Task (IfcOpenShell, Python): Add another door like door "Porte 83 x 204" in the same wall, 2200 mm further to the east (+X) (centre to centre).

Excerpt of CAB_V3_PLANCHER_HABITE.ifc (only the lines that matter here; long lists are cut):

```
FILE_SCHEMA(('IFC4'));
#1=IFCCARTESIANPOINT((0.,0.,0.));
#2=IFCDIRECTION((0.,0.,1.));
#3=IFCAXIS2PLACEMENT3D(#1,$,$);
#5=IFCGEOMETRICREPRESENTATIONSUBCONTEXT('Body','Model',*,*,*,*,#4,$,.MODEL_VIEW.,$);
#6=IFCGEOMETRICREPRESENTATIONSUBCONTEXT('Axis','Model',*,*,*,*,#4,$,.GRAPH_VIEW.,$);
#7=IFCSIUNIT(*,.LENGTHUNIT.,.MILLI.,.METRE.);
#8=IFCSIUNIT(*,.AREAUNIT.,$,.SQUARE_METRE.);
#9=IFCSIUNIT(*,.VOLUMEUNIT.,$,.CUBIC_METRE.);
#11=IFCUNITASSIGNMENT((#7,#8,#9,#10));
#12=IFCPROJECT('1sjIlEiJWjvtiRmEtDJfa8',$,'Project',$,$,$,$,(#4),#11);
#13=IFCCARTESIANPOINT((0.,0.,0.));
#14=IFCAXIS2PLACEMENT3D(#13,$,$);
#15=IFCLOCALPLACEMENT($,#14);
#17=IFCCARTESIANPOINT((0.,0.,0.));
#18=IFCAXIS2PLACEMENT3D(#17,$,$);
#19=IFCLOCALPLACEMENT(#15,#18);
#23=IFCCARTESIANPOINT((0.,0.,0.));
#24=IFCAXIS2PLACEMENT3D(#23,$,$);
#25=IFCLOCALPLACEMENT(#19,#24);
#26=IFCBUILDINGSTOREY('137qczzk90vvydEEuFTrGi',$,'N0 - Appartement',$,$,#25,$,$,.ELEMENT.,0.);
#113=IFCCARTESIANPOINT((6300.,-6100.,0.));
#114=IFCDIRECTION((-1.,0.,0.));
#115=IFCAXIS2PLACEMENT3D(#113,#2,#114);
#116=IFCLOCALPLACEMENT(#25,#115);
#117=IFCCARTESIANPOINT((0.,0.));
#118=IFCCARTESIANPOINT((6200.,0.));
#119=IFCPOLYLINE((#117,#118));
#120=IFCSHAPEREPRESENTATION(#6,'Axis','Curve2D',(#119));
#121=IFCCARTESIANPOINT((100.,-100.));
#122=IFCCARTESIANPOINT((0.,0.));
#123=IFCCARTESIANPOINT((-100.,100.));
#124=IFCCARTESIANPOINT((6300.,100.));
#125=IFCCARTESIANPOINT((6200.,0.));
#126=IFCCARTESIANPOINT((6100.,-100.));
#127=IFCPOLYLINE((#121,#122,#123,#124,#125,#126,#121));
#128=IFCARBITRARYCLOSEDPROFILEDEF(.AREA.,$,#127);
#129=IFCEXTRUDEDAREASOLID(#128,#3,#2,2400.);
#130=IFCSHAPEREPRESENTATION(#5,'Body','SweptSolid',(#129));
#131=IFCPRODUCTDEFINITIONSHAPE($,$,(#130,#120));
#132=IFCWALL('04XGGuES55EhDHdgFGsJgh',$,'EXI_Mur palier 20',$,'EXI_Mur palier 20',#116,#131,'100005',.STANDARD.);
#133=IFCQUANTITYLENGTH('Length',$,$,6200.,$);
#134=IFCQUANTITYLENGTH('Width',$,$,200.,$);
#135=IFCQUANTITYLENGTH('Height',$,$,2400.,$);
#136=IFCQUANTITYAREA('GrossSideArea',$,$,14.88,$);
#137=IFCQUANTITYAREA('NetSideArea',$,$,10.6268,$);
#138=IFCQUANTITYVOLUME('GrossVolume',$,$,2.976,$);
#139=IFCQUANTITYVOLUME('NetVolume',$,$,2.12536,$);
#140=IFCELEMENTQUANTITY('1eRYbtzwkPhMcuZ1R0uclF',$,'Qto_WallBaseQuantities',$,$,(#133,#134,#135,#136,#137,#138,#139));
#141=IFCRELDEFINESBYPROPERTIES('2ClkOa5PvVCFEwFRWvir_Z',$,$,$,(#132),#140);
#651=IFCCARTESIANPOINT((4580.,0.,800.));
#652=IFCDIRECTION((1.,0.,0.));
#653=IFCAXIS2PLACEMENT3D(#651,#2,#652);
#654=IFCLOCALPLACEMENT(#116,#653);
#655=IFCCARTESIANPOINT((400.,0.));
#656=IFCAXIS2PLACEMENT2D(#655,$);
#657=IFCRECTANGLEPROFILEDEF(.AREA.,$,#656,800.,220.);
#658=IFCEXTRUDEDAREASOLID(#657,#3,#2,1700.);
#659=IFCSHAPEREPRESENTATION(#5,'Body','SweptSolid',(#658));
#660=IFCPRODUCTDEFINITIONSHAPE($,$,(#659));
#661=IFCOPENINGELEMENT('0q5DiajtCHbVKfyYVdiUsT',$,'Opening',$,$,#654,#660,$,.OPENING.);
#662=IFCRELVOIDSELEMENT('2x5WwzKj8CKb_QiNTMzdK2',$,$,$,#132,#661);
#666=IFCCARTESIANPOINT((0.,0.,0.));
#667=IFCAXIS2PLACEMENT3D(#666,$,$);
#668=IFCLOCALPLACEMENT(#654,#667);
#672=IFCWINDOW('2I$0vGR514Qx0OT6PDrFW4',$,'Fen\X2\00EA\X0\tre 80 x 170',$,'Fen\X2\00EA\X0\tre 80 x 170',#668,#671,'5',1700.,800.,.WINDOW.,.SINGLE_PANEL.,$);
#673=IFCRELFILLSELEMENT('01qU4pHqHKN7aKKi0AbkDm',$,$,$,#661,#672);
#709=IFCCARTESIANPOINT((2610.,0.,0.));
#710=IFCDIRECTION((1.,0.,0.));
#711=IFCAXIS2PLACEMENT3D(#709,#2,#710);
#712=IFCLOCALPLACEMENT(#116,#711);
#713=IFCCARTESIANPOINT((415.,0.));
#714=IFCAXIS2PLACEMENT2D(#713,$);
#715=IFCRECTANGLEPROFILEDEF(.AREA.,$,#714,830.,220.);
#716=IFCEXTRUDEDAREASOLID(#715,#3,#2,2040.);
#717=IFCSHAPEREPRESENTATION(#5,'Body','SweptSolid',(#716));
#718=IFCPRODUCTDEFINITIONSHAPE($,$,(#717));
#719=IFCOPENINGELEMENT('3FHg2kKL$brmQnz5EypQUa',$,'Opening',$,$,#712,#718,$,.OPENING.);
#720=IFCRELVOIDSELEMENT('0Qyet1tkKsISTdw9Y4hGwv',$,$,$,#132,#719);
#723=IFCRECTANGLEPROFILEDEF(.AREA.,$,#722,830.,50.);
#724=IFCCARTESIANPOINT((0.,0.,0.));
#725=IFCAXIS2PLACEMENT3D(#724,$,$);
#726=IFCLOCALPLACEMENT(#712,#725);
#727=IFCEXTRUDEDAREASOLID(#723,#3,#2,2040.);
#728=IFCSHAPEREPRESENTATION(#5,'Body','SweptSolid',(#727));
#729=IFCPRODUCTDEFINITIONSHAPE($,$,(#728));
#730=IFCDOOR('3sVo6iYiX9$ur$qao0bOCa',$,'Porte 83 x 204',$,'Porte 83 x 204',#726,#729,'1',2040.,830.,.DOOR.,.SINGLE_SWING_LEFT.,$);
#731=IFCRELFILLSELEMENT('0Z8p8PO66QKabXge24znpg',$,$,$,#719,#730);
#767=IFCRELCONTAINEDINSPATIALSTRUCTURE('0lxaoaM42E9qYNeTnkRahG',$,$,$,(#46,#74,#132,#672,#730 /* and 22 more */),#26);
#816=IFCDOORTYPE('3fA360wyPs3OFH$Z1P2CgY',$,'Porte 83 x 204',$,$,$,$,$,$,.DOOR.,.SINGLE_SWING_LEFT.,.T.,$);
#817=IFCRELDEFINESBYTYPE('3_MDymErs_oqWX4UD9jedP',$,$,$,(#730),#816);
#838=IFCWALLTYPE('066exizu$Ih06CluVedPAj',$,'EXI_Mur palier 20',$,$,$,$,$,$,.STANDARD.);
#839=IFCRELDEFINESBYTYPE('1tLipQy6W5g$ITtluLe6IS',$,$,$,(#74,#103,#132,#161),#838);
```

```python
import ifcopenshell
import ifcopenshell.api.feature
import ifcopenshell.api.geometry
import ifcopenshell.api.pset
import ifcopenshell.api.root
import ifcopenshell.geom
import ifcopenshell.util.element
import ifcopenshell.util.placement
import ifcopenshell.util.shape
import ifcopenshell.util.unit

model = ifcopenshell.open("CAB_V3_PLANCHER_HABITE.ifc")
unit_scale = ifcopenshell.util.unit.calculate_unit_scale(model)
area_scale = ifcopenshell.util.unit.calculate_unit_scale(model, "AREAUNIT")
volume_scale = ifcopenshell.util.unit.calculate_unit_scale(model, "VOLUMEUNIT")
settings = ifcopenshell.geom.settings()


def volume(element):
    """Net volume in cubic metres, openings subtracted."""
    shape = ifcopenshell.geom.create_shape(settings, element)
    return ifcopenshell.util.shape.get_volume(shape.geometry)


door = model.by_guid("3sVo6iYiX9$ur$qao0bOCa")
opening = door.FillsVoids[0].RelatingOpeningElement
wall = opening.VoidsElements[0].RelatingBuildingElement
before = volume(wall)
shift = ifcopenshell.util.placement.get_local_placement(wall.ObjectPlacement)[:3, 0] * -2.2 / unit_scale

# copy_class copies the void relationship, type, container and properties, but no geometry.
new_opening = ifcopenshell.api.root.copy_class(model, product=opening)
new_opening.Representation = ifcopenshell.util.element.copy_deep(
    model, opening.Representation, exclude=["IfcGeometricRepresentationContext", "IfcRepresentationMap"]
)
new_door = ifcopenshell.api.root.copy_class(model, product=door)
new_door.Representation = ifcopenshell.util.element.copy_deep(
    model, door.Representation, exclude=["IfcGeometricRepresentationContext", "IfcRepresentationMap"]
)
new_door.Tag = None
ifcopenshell.api.feature.add_filling(model, opening=new_opening, element=new_door)

for old, new in ((opening, new_opening), (door, new_door)):
    matrix = ifcopenshell.util.placement.get_local_placement(old.ObjectPlacement)
    matrix[:3, 3] += shift
    ifcopenshell.api.geometry.edit_object_placement(model, product=new, matrix=matrix, is_si=False)

after = volume(wall)
thickness = 0.2  # wall thickness in metres

# Update the wall's stored quantities.
qto = model.by_id(ifcopenshell.util.element.get_pset(wall, "Qto_WallBaseQuantities", should_inherit=False)["id"])
ifcopenshell.api.pset.edit_qto(model, qto=qto, properties={
    "NetSideArea": after / thickness / area_scale,
    "NetVolume": after / volume_scale,
})

print(f"wall volume {before:.3f} -> {after:.3f} m3")

model.write("CAB_V3_PLANCHER_HABITE_rev.ifc")
```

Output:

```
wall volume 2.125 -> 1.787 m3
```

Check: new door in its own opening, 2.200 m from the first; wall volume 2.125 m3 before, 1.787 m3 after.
